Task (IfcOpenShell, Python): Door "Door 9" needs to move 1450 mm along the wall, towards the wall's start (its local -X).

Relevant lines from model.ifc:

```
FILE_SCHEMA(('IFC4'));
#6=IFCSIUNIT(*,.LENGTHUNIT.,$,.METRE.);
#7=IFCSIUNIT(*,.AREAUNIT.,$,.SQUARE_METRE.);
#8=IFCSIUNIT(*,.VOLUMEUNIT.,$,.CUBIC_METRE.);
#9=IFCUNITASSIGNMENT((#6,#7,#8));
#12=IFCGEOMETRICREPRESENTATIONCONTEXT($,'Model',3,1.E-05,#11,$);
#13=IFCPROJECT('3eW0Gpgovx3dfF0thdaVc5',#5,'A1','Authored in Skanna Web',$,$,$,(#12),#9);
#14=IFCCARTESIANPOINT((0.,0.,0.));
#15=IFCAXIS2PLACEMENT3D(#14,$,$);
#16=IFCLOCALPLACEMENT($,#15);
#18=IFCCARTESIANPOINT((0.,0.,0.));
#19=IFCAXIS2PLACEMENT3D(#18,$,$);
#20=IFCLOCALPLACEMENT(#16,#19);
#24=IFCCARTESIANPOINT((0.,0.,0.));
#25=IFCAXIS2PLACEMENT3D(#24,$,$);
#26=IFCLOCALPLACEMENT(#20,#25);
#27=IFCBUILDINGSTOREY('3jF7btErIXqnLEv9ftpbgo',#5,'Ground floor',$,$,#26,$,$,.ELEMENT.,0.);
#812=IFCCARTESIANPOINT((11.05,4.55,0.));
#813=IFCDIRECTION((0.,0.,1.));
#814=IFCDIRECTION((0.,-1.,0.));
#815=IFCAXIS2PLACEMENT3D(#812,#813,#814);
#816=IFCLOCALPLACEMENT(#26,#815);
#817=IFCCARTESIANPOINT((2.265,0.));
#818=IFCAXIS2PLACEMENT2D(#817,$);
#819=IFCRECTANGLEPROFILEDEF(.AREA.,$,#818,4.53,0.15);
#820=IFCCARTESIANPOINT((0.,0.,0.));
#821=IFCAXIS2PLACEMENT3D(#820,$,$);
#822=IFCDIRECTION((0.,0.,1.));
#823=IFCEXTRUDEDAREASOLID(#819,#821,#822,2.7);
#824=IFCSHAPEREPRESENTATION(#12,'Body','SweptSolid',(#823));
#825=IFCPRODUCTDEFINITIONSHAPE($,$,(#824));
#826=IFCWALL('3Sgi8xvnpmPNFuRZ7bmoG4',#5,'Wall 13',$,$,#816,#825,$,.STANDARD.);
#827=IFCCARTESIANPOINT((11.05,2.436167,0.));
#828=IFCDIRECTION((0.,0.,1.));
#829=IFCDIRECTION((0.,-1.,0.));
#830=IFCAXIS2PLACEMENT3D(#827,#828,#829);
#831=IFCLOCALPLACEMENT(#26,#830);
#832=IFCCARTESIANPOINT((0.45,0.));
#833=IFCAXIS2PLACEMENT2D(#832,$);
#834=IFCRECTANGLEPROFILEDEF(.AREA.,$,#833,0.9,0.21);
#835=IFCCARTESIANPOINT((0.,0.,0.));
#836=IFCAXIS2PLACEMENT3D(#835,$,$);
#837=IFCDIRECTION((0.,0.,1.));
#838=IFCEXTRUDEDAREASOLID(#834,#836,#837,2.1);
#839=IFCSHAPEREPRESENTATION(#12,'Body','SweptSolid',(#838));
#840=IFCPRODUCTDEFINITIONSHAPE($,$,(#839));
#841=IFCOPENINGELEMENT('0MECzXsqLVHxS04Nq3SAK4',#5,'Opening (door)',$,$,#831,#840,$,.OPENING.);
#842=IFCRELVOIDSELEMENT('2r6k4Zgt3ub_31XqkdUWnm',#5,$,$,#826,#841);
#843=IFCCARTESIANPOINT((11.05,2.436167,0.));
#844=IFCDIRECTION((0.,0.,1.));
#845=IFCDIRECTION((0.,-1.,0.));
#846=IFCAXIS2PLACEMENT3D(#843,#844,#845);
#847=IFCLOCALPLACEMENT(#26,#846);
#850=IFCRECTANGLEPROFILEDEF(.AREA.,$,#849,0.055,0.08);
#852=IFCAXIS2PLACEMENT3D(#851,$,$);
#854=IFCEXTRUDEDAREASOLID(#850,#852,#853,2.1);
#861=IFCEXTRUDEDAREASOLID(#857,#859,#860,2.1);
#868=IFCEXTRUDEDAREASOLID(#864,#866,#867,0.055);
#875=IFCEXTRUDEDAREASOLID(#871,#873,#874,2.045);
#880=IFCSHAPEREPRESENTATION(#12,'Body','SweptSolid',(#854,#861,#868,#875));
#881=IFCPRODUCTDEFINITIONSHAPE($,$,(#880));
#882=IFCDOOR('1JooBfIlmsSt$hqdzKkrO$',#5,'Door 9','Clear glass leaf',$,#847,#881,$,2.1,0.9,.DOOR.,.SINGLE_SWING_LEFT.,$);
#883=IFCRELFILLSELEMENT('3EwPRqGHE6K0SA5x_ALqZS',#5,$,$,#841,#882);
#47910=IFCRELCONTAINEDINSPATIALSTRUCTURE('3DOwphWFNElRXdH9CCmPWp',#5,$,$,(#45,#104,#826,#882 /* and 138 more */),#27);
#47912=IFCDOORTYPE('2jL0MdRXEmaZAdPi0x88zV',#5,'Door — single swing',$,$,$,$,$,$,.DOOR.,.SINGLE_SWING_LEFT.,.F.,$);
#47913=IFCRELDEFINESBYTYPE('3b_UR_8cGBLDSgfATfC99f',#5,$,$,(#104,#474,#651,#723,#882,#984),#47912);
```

```python
import ifcopenshell
import ifcopenshell.api.geometry
import ifcopenshell.util.placement

model = ifcopenshell.open("model.ifc")

door = model.by_id(882)
opening = door.FillsVoids[0].RelatingOpeningElement
wall = opening.VoidsElements[0].RelatingBuildingElement

wall_matrix = ifcopenshell.util.placement.get_local_placement(wall.ObjectPlacement)
shift = wall_matrix[:3, 0] * -1.45
before = ifcopenshell.util.placement.get_local_placement(door.ObjectPlacement)[:3, 3].copy()

# The door is not placed relative to its opening, so move both.
for product in (opening, door):
    matrix = ifcopenshell.util.placement.get_local_placement(product.ObjectPlacement)
    matrix[:3, 3] += shift
    ifcopenshell.api.geometry.edit_object_placement(model, product=product, matrix=matrix, is_si=False)

after = ifcopenshell.util.placement.get_local_placement(door.ObjectPlacement)[:3, 3]
print("door moved by", (after - before).round(3) + 0.0)

model.write("model_edited.ifc")
```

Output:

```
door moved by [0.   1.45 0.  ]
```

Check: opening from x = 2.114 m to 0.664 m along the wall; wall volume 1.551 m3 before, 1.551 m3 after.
